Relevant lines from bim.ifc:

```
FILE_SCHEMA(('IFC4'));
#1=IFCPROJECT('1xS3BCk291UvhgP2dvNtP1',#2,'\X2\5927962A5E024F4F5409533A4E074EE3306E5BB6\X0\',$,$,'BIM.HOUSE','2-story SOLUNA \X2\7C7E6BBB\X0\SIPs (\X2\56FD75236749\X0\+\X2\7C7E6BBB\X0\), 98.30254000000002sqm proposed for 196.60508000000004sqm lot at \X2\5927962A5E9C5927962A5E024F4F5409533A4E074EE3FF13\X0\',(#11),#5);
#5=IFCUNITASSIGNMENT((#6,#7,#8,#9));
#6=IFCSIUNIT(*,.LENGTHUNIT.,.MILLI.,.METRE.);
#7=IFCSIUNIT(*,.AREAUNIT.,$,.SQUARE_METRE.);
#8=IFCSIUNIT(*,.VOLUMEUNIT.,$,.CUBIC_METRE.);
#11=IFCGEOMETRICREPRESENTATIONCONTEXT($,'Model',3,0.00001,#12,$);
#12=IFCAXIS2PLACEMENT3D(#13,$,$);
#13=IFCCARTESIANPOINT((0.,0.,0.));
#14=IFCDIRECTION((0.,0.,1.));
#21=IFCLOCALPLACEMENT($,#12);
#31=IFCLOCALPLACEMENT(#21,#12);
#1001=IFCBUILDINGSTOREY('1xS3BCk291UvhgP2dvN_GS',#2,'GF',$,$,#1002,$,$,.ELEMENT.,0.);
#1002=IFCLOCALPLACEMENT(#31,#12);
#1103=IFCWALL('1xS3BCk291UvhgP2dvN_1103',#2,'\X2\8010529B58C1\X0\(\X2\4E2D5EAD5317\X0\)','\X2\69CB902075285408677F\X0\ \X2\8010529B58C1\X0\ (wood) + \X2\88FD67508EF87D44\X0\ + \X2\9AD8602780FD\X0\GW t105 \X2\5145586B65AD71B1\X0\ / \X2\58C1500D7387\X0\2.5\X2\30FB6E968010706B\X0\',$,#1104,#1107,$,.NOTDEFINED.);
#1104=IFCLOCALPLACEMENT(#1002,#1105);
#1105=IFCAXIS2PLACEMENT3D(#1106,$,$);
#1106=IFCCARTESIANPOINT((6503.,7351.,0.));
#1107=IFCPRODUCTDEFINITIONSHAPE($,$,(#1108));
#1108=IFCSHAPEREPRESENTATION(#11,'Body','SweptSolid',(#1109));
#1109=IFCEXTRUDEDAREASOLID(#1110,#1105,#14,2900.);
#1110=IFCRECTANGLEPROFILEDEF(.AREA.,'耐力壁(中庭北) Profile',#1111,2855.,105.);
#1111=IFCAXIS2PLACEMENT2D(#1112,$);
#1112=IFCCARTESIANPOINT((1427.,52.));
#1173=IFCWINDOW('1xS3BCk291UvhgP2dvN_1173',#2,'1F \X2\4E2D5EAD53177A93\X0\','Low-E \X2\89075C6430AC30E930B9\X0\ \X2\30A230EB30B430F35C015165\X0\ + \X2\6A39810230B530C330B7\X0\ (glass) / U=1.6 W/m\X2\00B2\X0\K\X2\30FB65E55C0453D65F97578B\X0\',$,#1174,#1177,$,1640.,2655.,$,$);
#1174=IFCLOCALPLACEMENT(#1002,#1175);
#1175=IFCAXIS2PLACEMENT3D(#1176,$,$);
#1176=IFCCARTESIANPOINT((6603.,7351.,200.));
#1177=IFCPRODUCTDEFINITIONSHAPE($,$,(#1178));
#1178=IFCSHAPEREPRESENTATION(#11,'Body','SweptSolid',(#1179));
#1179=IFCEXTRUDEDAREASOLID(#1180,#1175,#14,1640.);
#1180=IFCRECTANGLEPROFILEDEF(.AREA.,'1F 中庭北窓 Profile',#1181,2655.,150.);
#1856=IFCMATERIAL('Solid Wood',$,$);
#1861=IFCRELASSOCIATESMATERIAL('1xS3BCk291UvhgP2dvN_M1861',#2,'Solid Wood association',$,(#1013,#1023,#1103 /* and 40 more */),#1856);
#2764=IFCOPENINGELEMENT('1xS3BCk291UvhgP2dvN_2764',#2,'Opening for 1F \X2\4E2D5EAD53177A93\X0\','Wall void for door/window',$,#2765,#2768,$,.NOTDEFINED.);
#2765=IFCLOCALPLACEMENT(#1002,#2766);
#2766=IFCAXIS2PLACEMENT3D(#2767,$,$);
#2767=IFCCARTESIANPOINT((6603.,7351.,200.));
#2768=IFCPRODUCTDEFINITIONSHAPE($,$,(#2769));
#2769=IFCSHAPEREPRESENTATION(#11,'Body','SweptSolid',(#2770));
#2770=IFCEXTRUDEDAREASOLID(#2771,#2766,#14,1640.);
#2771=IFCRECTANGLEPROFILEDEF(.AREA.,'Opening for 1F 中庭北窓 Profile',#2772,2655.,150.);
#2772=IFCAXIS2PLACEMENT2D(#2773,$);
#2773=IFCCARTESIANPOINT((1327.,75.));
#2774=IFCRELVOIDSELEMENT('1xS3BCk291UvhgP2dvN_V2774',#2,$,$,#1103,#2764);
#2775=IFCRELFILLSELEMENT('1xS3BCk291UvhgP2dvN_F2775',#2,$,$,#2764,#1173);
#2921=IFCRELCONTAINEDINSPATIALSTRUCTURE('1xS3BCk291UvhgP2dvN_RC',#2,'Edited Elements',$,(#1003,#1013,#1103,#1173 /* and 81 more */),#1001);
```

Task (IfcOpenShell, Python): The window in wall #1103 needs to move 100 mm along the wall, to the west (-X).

```python
import ifcopenshell
import ifcopenshell.api.geometry
import ifcopenshell.util.placement

model = ifcopenshell.open("bim.ifc")

window = model.by_id(1173)
opening = window.FillsVoids[0].RelatingOpeningElement
wall = opening.VoidsElements[0].RelatingBuildingElement

wall_matrix = ifcopenshell.util.placement.get_local_placement(wall.ObjectPlacement)
shift = wall_matrix[:3, 0] * -100.0
before = ifcopenshell.util.placement.get_local_placement(window.ObjectPlacement)[:3, 3].copy()

# The window is not placed relative to its opening, so move both.
for product in (opening, window):
    matrix = ifcopenshell.util.placement.get_local_placement(product.ObjectPlacement)
    matrix[:3, 3] += shift
    ifcopenshell.api.geometry.edit_object_placement(model, product=product, matrix=matrix, is_si=False)

after = ifcopenshell.util.placement.get_local_placement(window.ObjectPlacement)[:3, 3]
print("window moved by", (after - before).round(3) + 0.0)

model.write("bim_rev.ifc")
```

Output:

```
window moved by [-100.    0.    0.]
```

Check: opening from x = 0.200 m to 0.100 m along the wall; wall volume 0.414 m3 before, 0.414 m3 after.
